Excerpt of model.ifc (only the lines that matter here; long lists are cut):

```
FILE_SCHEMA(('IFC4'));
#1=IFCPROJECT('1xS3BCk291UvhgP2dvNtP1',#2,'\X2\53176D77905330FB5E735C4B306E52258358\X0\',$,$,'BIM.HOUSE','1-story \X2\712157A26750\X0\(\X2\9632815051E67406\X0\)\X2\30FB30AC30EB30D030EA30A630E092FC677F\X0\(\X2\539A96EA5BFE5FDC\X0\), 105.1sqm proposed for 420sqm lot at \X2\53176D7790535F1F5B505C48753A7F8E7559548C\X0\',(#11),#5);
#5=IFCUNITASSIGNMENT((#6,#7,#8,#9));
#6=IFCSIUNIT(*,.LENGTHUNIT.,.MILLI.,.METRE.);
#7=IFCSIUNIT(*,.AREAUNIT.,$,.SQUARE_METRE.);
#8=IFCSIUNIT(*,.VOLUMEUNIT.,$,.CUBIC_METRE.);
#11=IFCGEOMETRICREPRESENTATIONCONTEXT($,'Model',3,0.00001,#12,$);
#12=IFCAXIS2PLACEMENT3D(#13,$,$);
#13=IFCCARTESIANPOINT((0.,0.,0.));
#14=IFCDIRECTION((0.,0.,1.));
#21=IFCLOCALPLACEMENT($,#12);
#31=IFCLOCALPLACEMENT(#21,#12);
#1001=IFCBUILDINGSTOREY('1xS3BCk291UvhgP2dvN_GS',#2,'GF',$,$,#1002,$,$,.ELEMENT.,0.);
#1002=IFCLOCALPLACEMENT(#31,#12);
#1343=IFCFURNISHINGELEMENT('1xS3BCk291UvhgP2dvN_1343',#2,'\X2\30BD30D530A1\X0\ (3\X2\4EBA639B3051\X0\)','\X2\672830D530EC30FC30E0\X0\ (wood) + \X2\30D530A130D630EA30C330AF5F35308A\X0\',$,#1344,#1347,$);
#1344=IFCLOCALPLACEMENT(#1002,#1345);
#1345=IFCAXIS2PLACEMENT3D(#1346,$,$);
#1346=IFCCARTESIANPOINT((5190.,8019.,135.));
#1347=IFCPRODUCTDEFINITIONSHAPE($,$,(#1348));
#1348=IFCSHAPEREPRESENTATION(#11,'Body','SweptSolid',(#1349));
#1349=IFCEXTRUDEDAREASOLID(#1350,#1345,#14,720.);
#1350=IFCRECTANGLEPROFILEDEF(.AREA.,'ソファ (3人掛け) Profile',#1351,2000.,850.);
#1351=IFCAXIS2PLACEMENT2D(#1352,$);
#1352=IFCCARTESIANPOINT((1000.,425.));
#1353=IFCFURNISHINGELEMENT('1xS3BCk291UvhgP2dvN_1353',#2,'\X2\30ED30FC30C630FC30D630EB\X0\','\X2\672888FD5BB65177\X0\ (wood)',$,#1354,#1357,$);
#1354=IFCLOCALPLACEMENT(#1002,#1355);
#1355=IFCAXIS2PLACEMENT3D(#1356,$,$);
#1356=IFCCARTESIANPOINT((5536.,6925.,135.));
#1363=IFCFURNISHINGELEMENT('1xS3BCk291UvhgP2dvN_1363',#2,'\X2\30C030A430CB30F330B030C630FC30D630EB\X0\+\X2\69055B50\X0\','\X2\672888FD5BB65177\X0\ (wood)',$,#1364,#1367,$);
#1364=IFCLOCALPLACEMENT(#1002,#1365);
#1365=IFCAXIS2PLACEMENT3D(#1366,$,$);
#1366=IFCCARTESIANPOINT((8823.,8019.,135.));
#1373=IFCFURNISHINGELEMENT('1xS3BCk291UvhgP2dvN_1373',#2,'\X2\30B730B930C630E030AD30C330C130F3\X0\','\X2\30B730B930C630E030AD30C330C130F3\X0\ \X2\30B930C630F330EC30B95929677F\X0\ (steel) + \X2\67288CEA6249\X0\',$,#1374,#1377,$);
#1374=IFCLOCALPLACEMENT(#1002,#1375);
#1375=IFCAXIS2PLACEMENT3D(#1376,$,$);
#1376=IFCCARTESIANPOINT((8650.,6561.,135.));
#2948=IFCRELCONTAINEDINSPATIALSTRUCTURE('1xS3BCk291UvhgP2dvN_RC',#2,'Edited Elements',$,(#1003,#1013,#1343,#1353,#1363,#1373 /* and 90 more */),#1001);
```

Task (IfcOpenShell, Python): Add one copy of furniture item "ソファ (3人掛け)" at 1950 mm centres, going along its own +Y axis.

```python
import ifcopenshell
import ifcopenshell.api.geometry
import ifcopenshell.api.root
import ifcopenshell.util.element
import ifcopenshell.util.placement
import ifcopenshell.util.unit

model = ifcopenshell.open("model.ifc")
unit_scale = ifcopenshell.util.unit.calculate_unit_scale(model)


def reuse_history(source, copy):
    """copy_class also copies each property set's owner history, people and application; keep the originals."""
    for rel in copy.IsDefinedBy:
        if rel.is_a("IfcRelDefinesByProperties") and (history := rel.RelatingPropertyDefinition.OwnerHistory):
            rel.RelatingPropertyDefinition.OwnerHistory = source.OwnerHistory
            ifcopenshell.util.element.remove_deep2(model, history)


source = model.by_guid("1xS3BCk291UvhgP2dvN_1343")
base = ifcopenshell.util.placement.get_local_placement(source.ObjectPlacement)
step = base[:3, 1] * 1.95 / unit_scale

for i in range(1, 2):
    copy = ifcopenshell.api.root.copy_class(model, product=source)
    copy.Representation = ifcopenshell.util.element.copy_deep(
        model, source.Representation, exclude=["IfcGeometricRepresentationContext", "IfcRepresentationMap"]
    )
    reuse_history(source, copy)
    matrix = base.copy()
    matrix[:3, 3] += i * step
    print("added at", matrix[:3, 3].round(3) + 0.0)
    ifcopenshell.api.geometry.edit_object_placement(model, product=copy, matrix=matrix, is_si=False)

model.write("model_updated.ifc")
```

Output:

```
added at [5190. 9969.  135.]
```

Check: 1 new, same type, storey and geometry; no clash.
